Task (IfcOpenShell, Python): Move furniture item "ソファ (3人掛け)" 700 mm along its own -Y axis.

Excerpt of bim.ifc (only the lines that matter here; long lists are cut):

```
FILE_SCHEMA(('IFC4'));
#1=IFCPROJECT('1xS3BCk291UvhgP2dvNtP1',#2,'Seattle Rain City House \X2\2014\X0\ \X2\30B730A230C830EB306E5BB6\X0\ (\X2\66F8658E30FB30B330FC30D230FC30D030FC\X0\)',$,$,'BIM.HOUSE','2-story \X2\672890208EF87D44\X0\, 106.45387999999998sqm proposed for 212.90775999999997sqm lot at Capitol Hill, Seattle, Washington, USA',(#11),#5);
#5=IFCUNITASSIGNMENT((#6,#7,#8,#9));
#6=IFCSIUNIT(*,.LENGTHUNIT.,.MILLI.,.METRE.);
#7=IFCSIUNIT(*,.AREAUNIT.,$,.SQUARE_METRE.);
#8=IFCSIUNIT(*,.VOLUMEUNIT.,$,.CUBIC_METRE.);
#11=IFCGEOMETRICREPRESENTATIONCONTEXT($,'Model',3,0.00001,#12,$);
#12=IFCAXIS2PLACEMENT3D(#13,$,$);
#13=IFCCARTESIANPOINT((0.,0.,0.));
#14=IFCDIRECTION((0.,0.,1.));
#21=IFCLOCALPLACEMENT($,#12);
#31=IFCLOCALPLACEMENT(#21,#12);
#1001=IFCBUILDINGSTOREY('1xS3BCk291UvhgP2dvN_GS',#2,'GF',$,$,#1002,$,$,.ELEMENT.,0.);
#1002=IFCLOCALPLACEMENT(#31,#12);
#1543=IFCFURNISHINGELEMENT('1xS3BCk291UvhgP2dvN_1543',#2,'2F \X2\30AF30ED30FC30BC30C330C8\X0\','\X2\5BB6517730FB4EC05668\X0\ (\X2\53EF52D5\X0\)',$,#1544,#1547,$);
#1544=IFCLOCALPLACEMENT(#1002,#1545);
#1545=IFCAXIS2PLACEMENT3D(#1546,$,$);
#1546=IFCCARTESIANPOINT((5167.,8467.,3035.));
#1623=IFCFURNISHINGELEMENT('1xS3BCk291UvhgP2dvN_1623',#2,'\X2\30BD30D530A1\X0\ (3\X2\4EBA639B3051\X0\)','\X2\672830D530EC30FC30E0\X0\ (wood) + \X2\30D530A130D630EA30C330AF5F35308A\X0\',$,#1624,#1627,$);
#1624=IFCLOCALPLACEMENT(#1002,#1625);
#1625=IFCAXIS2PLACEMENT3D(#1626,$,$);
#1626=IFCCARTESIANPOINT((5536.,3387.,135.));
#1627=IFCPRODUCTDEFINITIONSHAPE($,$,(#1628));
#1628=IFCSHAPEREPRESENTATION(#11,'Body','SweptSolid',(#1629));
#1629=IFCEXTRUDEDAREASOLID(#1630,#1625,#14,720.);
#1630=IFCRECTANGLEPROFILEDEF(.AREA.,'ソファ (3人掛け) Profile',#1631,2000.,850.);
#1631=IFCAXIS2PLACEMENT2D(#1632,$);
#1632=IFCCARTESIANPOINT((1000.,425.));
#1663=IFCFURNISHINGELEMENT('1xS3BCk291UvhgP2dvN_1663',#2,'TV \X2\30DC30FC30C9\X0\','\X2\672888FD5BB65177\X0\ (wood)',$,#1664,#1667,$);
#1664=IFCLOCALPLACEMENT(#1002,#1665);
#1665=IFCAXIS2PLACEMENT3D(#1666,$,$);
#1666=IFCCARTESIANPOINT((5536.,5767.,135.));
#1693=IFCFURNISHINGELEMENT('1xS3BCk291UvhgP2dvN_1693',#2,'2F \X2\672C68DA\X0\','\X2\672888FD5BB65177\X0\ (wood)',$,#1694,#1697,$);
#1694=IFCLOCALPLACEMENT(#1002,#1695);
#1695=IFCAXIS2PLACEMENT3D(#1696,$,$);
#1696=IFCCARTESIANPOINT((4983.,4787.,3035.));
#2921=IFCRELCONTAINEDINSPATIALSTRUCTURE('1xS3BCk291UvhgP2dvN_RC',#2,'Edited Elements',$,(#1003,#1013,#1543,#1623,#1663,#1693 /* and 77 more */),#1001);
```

```python
import ifcopenshell
import ifcopenshell.api.geometry
import ifcopenshell.util.placement

model = ifcopenshell.open("bim.ifc")

item = model.by_guid("1xS3BCk291UvhgP2dvN_1623")
matrix = ifcopenshell.util.placement.get_local_placement(item.ObjectPlacement)
matrix[:3, 3] -= matrix[:3, 1] * 700.0
ifcopenshell.api.geometry.edit_object_placement(model, product=item, matrix=matrix, is_si=False)

print(ifcopenshell.util.placement.get_local_placement(item.ObjectPlacement).round(3) + 0.0)

model.write("bim_edited.ifc")
```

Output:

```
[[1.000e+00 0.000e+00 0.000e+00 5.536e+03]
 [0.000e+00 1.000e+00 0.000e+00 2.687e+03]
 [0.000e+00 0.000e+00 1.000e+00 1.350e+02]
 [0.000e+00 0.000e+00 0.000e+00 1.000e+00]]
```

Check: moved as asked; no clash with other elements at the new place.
